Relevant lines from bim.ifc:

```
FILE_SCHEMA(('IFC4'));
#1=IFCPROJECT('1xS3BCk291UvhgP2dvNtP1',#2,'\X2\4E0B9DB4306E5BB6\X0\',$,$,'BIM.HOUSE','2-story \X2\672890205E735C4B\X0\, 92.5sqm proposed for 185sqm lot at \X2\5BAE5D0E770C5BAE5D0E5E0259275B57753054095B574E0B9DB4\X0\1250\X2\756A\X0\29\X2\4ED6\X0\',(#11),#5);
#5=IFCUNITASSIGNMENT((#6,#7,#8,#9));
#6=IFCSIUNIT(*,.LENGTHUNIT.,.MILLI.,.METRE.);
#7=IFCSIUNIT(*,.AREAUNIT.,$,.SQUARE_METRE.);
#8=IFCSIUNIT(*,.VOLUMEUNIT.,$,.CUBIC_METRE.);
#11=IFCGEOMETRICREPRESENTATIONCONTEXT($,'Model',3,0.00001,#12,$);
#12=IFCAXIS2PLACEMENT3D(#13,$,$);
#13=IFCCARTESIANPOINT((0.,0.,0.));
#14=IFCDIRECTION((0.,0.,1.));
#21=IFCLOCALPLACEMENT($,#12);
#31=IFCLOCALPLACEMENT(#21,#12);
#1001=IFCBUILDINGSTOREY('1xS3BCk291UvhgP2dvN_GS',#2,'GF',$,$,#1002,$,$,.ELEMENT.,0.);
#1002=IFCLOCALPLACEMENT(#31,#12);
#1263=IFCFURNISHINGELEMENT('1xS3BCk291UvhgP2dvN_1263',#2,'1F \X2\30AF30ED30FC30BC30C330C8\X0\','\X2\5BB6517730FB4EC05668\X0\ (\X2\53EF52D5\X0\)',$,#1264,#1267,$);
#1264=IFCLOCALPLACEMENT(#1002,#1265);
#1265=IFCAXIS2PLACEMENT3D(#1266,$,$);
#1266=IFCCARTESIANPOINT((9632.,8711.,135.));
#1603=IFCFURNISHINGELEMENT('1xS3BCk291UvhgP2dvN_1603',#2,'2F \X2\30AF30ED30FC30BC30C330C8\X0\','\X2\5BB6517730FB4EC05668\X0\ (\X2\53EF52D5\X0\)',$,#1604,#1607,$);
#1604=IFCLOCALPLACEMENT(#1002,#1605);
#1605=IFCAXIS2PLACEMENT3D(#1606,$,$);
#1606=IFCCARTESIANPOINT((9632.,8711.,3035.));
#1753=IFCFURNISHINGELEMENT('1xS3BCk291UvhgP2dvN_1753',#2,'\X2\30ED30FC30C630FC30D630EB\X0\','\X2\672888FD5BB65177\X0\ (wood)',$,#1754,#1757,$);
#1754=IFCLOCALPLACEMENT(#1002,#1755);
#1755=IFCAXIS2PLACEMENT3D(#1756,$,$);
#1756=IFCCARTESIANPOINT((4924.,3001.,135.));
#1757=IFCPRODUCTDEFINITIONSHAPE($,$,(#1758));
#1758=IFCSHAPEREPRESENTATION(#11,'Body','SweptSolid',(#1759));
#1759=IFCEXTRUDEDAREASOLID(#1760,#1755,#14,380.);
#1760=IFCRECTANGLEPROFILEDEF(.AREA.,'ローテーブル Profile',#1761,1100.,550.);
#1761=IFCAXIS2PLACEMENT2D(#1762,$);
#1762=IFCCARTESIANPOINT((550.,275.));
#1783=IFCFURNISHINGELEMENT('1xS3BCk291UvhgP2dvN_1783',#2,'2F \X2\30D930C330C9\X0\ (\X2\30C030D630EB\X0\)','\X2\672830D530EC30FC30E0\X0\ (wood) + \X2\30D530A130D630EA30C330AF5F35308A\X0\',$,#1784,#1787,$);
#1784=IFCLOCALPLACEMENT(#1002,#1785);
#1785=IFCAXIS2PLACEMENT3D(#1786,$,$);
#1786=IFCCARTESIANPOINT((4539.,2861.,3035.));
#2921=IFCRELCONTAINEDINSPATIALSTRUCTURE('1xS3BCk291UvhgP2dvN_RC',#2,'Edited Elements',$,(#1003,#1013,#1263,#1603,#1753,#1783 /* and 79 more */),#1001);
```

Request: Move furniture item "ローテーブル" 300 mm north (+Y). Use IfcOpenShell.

```python
import ifcopenshell
import ifcopenshell.api.geometry
import ifcopenshell.util.placement
import ifcopenshell.util.unit

model = ifcopenshell.open("bim.ifc")
unit_scale = ifcopenshell.util.unit.calculate_unit_scale(model)

item = model.by_guid("1xS3BCk291UvhgP2dvN_1753")
matrix = ifcopenshell.util.placement.get_local_placement(item.ObjectPlacement)
matrix[1, 3] += 0.3 / unit_scale
ifcopenshell.api.geometry.edit_object_placement(model, product=item, matrix=matrix, is_si=False)

print(ifcopenshell.util.placement.get_local_placement(item.ObjectPlacement).round(3) + 0.0)

model.write("bim_updated.ifc")
```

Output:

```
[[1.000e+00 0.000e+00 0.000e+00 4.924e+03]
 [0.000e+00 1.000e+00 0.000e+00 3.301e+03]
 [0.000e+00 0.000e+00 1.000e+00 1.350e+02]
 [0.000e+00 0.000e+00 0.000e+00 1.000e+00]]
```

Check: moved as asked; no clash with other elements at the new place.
